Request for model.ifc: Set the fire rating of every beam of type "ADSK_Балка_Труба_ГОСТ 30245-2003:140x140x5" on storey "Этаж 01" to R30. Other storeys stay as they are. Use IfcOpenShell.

First a look at what the model holds.

```python
import ifcopenshell
import ifcopenshell.util.element

model = ifcopenshell.open("model.ifc")
print(model.schema)
storey = next(s for s in model.by_type("IfcBuildingStorey") if s.Name == "Этаж 01")
beams = [e for e in ifcopenshell.util.element.get_decomposition(storey) if e.is_a("IfcBeam")]
seen = {}
for e in beams:
    element_type = ifcopenshell.util.element.get_type(e)
    key = (element_type.Name if element_type != e and element_type else None, ifcopenshell.util.element.get_pset(e, "Pset_BeamCommon", "FireRating"))
    seen[key] = seen.get(key, 0) + 1
for (name, value), count in sorted(seen.items(), key=str):
    print(count, "x", name, "|", value)
```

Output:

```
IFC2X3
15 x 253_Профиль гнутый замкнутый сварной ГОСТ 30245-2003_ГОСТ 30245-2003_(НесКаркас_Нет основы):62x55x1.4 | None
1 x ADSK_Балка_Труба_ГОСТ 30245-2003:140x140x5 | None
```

```python
import ifcopenshell
import ifcopenshell.api.pset
import ifcopenshell.util.element

model = ifcopenshell.open("model.ifc")

storey = next(s for s in model.by_type("IfcBuildingStorey") if s.Name == "Этаж 01")
beams = [e for e in ifcopenshell.util.element.get_decomposition(storey) if e.is_a("IfcBeam")]

count = 0
for e in beams:
    element_type = ifcopenshell.util.element.get_type(e)
    if element_type in (None, e) or element_type.Name != "ADSK_Балка_Труба_ГОСТ 30245-2003:140x140x5":
        continue
    # add_pset returns the element's existing set when there is one.
    pset = ifcopenshell.api.pset.add_pset(model, product=e, name="Pset_BeamCommon")
    ifcopenshell.api.pset.edit_pset(model, pset=pset, properties={"FireRating": "R30"})
    count += 1

print(count, "beams updated")

model.write("model_rev.ifc")
```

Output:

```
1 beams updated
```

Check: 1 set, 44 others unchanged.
